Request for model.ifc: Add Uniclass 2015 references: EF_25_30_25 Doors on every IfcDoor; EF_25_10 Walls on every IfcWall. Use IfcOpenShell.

First a look at what the model holds.

```python
import ifcopenshell

model = ifcopenshell.open("model.ifc")
print(model.schema)
print("classifications:", [c.Name for c in model.by_type("IfcClassification")])
for ifc_class in ("IfcDoor", "IfcRoof", "IfcStair", "IfcWall", "IfcWindow"):
    print(ifc_class, len(model.by_type(ifc_class)))
```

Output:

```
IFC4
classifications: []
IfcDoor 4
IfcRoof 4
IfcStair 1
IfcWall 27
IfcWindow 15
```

```python
import ifcopenshell
import ifcopenshell.api.classification

model = ifcopenshell.open("model.ifc")

system = ifcopenshell.api.classification.add_classification(model, classification="Uniclass 2015")

codes = {
    "IfcDoor": ("EF_25_30_25", "Doors"),
    "IfcWall": ("EF_25_10", "Walls"),
}
for ifc_class, (code, name) in codes.items():
    products = model.by_type(ifc_class)
    ifcopenshell.api.classification.add_reference(
        model, products=products, classification=system, identification=code, name=name
    )
    print(code, len(products))

model.write("model_rev.ifc")
```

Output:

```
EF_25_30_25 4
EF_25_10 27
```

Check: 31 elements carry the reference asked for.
